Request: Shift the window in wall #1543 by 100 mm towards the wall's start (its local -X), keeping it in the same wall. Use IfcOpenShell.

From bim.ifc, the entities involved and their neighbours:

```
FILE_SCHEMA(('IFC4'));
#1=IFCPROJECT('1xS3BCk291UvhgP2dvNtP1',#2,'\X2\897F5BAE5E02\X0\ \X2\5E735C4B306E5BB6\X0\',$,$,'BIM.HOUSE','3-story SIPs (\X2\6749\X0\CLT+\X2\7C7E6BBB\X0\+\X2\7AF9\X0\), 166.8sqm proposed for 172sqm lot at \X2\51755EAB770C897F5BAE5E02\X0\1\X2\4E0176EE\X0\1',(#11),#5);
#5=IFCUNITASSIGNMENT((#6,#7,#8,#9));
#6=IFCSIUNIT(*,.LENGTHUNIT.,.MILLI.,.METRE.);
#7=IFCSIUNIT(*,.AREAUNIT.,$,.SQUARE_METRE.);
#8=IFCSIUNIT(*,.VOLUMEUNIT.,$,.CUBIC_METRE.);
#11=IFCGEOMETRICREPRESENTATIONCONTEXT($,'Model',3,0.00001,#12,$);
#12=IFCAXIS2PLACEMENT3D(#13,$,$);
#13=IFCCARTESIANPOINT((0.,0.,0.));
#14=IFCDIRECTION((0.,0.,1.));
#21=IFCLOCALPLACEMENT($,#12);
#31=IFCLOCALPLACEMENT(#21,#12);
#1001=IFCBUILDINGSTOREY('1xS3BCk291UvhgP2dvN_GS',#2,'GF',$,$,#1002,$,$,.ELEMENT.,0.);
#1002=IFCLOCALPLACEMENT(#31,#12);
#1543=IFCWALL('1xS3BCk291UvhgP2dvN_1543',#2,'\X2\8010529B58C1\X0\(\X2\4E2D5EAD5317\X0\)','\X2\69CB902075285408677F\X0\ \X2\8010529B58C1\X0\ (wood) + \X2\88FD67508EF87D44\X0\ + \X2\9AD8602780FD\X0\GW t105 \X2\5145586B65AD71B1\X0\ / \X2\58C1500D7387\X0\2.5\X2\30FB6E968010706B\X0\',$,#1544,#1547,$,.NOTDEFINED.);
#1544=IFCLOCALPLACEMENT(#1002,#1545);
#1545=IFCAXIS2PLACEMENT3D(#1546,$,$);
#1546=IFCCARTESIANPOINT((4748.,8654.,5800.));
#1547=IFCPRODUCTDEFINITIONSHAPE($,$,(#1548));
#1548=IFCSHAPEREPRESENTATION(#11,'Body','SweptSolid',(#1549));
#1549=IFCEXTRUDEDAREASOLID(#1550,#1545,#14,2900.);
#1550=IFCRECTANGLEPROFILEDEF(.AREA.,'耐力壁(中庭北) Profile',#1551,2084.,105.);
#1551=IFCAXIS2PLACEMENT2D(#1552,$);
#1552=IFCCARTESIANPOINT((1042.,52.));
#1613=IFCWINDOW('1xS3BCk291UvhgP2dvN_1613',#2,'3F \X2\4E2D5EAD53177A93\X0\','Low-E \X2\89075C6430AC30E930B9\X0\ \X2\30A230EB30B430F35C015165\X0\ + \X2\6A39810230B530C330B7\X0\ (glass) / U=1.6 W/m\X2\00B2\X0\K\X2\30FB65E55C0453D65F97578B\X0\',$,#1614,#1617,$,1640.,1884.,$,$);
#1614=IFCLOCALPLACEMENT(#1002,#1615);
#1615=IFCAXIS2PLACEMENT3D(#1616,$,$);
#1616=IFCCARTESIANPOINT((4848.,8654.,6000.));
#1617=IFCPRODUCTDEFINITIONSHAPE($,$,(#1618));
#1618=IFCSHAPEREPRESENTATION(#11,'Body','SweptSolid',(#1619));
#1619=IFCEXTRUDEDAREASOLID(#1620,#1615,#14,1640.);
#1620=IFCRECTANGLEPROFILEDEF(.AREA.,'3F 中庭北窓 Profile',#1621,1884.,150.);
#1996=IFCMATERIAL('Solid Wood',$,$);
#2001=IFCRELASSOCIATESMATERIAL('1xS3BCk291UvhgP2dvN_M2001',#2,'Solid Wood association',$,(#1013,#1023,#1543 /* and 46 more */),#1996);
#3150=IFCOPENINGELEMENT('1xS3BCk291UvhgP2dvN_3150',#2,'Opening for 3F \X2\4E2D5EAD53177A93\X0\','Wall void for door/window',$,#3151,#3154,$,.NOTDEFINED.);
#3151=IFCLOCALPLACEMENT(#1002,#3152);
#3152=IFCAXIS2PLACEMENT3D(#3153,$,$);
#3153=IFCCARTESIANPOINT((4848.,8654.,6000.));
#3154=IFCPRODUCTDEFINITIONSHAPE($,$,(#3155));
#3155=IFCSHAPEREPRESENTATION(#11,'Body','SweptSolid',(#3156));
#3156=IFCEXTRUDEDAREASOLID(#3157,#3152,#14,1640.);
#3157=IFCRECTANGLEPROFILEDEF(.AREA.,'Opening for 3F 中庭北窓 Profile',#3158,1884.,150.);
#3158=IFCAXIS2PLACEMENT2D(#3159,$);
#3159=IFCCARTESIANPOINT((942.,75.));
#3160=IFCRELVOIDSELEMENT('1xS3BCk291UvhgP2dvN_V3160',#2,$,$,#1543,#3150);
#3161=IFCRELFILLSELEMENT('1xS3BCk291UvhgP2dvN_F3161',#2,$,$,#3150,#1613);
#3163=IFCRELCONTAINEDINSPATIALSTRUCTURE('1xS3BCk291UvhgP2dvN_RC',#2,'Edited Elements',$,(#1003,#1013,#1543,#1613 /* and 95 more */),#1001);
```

```python
import ifcopenshell
import ifcopenshell.api.geometry
import ifcopenshell.util.placement

model = ifcopenshell.open("bim.ifc")

window = model.by_id(1613)
opening = window.FillsVoids[0].RelatingOpeningElement
wall = opening.VoidsElements[0].RelatingBuildingElement

wall_matrix = ifcopenshell.util.placement.get_local_placement(wall.ObjectPlacement)
shift = wall_matrix[:3, 0] * -100.0
before = ifcopenshell.util.placement.get_local_placement(window.ObjectPlacement)[:3, 3].copy()

# The window is not placed relative to its opening, so move both.
for product in (opening, window):
    matrix = ifcopenshell.util.placement.get_local_placement(product.ObjectPlacement)
    matrix[:3, 3] += shift
    ifcopenshell.api.geometry.edit_object_placement(model, product=product, matrix=matrix, is_si=False)

after = ifcopenshell.util.placement.get_local_placement(window.ObjectPlacement)[:3, 3]
print("window moved by", (after - before).round(3) + 0.0)

model.write("bim_edited.ifc")
```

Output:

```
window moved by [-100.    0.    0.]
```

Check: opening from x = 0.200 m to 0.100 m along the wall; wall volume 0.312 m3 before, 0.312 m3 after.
